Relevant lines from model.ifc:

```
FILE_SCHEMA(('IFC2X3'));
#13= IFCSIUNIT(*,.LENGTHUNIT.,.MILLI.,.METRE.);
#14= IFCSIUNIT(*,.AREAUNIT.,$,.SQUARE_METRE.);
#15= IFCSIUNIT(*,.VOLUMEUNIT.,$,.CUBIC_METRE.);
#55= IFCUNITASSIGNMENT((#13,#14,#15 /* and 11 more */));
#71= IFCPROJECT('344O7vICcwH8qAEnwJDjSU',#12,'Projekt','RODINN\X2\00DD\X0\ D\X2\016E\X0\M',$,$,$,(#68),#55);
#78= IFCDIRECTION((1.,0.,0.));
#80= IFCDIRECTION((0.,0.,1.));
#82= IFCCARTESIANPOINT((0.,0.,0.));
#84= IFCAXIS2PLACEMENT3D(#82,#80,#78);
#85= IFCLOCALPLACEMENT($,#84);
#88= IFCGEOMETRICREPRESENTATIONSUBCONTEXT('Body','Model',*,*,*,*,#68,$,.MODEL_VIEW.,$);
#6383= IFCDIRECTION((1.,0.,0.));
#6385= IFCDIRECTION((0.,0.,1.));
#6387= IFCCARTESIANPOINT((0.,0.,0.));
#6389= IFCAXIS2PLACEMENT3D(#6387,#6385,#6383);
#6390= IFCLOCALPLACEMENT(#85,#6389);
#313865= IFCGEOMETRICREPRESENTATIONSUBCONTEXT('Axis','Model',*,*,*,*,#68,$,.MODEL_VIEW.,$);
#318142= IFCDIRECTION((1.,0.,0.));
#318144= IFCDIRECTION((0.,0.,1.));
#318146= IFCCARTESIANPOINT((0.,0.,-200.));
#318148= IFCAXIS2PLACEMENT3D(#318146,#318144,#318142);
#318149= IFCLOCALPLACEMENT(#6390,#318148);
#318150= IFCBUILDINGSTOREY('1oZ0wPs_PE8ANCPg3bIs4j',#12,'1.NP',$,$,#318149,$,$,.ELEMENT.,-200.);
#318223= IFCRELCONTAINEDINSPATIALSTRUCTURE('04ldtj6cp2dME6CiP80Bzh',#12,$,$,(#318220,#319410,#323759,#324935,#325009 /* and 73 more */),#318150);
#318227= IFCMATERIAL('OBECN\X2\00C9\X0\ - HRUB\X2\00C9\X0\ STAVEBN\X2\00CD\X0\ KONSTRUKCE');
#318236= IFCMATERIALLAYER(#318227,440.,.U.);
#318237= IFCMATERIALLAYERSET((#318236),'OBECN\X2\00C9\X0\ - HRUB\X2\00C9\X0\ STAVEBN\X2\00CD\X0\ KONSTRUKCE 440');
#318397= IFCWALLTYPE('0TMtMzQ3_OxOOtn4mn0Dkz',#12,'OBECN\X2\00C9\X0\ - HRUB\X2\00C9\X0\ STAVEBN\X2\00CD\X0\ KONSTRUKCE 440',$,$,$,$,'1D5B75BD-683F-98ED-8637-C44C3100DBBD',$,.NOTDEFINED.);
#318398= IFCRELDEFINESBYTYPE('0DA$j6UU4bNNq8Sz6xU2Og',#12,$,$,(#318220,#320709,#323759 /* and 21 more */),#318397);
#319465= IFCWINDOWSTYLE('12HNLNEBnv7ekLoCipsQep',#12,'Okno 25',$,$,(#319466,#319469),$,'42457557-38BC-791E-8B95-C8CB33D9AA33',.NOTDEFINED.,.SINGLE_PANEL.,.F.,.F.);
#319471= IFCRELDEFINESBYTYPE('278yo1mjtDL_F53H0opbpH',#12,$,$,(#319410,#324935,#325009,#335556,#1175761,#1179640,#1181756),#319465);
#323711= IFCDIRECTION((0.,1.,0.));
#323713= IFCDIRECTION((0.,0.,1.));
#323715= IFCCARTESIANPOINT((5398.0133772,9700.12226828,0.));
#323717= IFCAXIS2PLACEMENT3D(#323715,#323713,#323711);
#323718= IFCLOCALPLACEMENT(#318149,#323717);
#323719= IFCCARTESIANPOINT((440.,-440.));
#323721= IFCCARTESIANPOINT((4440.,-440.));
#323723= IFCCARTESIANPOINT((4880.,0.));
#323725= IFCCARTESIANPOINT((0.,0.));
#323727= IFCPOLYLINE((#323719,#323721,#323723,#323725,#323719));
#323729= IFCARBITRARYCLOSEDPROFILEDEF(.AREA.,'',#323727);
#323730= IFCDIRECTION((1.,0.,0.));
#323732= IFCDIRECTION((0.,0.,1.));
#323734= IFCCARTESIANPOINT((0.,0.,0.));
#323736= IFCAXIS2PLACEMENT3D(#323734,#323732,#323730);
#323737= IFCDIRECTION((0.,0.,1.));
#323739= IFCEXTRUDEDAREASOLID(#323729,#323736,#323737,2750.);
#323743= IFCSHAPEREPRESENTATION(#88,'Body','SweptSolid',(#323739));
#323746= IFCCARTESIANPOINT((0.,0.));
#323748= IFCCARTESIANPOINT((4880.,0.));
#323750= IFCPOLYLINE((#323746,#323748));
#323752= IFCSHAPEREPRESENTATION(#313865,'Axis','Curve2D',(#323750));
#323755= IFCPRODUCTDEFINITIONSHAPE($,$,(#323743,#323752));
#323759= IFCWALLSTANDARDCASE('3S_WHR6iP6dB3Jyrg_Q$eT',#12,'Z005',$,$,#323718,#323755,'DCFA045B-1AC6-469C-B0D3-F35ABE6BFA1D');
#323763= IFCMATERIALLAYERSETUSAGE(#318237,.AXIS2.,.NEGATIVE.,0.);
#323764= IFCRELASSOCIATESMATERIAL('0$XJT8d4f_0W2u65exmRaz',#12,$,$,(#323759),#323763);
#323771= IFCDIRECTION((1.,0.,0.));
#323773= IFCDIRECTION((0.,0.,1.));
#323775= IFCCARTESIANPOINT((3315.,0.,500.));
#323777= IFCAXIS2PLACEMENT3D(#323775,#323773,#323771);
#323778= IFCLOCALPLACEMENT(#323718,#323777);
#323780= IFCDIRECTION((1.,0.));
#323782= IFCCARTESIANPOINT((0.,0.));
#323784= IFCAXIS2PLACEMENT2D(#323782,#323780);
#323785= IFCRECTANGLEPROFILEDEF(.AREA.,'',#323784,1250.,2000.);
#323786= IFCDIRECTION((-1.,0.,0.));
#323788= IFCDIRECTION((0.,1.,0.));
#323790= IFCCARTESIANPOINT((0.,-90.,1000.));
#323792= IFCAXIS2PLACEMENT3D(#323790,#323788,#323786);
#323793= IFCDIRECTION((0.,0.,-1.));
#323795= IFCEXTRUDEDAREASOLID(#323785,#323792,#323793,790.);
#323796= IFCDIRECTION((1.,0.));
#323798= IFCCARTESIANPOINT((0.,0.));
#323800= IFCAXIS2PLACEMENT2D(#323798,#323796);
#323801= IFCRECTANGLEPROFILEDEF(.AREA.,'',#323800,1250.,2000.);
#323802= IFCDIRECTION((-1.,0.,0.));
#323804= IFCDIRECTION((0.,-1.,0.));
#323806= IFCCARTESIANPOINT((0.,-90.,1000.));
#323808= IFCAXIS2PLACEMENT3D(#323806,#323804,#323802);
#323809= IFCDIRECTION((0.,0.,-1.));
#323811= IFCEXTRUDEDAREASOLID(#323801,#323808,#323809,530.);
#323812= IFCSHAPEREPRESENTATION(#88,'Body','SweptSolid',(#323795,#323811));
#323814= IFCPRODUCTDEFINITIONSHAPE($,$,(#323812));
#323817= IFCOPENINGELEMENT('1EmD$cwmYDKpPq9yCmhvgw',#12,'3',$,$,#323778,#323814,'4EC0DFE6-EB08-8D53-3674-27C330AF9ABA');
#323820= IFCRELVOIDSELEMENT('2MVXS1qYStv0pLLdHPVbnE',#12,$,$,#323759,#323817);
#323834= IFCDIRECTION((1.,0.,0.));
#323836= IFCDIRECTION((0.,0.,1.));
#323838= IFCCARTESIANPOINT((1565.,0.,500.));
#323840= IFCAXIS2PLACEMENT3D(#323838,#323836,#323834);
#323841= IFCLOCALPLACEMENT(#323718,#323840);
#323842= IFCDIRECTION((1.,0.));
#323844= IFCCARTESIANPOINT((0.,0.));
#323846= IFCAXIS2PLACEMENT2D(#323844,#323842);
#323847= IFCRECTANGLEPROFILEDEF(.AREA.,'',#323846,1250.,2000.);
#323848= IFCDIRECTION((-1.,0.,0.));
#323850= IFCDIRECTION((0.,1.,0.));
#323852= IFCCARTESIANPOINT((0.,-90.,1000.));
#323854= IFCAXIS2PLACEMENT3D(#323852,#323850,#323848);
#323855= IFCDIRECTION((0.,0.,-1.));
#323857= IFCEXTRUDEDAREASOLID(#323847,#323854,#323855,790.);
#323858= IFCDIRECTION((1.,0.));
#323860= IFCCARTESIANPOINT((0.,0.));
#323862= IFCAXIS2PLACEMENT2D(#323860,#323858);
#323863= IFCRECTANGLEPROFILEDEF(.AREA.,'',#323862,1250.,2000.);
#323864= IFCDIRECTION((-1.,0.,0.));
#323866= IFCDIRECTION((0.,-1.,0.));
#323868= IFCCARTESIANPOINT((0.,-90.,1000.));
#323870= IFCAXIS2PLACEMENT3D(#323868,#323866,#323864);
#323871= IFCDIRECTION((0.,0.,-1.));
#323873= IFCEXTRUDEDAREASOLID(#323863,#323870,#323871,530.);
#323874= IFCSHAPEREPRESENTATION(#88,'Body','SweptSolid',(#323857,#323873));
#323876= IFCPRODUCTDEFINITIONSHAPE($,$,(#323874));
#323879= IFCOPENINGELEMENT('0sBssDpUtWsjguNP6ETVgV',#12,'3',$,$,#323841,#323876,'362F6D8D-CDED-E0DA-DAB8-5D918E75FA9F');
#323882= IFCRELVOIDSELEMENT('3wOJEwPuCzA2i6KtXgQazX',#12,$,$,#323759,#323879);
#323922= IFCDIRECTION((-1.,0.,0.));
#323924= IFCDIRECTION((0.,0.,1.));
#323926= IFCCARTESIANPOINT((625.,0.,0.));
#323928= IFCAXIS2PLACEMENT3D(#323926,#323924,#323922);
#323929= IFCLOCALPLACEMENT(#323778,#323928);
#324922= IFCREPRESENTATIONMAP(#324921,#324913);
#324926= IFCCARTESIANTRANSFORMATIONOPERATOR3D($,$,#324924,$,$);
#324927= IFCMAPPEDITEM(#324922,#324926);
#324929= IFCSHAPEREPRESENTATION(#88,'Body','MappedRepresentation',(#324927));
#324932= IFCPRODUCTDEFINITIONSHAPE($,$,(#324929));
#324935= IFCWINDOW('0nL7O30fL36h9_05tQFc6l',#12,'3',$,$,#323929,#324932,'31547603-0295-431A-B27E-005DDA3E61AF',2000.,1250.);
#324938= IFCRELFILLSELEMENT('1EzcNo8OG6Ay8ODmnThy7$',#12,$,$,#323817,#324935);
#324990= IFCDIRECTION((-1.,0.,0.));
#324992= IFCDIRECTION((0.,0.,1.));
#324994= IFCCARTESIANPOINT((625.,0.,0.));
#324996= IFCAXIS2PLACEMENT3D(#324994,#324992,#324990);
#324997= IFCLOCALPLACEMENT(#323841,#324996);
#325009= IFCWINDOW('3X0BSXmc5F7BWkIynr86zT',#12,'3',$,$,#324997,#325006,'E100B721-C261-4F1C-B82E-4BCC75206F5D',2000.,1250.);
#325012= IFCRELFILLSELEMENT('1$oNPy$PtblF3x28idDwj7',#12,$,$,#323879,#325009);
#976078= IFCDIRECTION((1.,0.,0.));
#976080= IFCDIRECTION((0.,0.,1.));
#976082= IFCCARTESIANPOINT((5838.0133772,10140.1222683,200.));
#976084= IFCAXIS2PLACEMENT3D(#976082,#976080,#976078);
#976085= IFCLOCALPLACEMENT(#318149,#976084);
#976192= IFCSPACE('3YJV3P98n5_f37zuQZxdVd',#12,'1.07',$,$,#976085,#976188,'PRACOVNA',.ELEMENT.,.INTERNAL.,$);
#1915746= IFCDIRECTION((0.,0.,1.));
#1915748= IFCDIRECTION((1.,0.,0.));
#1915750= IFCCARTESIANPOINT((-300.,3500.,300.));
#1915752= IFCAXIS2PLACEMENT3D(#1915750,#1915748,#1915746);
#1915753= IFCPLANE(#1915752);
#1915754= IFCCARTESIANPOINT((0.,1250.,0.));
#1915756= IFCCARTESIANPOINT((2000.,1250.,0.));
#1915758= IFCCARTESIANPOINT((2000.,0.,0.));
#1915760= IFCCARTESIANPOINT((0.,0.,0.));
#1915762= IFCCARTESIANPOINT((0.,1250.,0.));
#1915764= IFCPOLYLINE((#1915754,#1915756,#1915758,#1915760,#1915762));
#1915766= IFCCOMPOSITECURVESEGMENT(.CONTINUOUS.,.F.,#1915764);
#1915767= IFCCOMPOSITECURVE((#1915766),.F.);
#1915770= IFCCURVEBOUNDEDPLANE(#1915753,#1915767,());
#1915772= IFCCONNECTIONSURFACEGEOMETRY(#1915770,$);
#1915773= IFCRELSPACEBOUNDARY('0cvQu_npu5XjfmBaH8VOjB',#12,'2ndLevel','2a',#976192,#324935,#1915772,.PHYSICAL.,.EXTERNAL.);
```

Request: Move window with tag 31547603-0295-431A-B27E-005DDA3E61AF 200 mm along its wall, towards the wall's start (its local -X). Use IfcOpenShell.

```python
import numpy as np
import ifcopenshell
import ifcopenshell.api.geometry
import ifcopenshell.util.placement

model = ifcopenshell.open("model.ifc")

window = model.by_guid("0nL7O30fL36h9_05tQFc6l")
opening = window.FillsVoids[0].RelatingOpeningElement
wall = opening.VoidsElements[0].RelatingBuildingElement

wall_matrix = ifcopenshell.util.placement.get_local_placement(wall.ObjectPlacement)
shift = wall_matrix[:3, 0] * -200.0
before = ifcopenshell.util.placement.get_local_placement(window.ObjectPlacement)[:3, 3].copy()

# The window is placed relative to its opening, so it follows when the opening moves.
matrix = ifcopenshell.util.placement.get_local_placement(opening.ObjectPlacement)
matrix[:3, 3] += shift
ifcopenshell.api.geometry.edit_object_placement(
    model, product=opening, matrix=matrix, is_si=False, should_transform_children=True
)

# Space boundary surfaces are stored in each space's coordinates; move them too.
for rel in window.ProvidesBoundaries:
    if not rel.ConnectionGeometry:
        continue
    surface = rel.ConnectionGeometry.SurfaceOnRelatingElement.BasisSurface
    space_matrix = ifcopenshell.util.placement.get_local_placement(rel.RelatingSpace.ObjectPlacement)
    point = np.array(surface.Position.Location.Coordinates) + space_matrix[:3, :3].T @ shift
    surface.Position = model.createIfcAxis2Placement3D(
        model.createIfcCartesianPoint(point.tolist()), surface.Position.Axis, surface.Position.RefDirection
    )

after = ifcopenshell.util.placement.get_local_placement(window.ObjectPlacement)[:3, 3]
print("window moved by", (after - before).round(3) + 0.0)

model.write("model_v2.ifc")
```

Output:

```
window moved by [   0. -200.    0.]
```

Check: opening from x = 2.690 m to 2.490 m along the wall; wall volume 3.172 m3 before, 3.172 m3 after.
